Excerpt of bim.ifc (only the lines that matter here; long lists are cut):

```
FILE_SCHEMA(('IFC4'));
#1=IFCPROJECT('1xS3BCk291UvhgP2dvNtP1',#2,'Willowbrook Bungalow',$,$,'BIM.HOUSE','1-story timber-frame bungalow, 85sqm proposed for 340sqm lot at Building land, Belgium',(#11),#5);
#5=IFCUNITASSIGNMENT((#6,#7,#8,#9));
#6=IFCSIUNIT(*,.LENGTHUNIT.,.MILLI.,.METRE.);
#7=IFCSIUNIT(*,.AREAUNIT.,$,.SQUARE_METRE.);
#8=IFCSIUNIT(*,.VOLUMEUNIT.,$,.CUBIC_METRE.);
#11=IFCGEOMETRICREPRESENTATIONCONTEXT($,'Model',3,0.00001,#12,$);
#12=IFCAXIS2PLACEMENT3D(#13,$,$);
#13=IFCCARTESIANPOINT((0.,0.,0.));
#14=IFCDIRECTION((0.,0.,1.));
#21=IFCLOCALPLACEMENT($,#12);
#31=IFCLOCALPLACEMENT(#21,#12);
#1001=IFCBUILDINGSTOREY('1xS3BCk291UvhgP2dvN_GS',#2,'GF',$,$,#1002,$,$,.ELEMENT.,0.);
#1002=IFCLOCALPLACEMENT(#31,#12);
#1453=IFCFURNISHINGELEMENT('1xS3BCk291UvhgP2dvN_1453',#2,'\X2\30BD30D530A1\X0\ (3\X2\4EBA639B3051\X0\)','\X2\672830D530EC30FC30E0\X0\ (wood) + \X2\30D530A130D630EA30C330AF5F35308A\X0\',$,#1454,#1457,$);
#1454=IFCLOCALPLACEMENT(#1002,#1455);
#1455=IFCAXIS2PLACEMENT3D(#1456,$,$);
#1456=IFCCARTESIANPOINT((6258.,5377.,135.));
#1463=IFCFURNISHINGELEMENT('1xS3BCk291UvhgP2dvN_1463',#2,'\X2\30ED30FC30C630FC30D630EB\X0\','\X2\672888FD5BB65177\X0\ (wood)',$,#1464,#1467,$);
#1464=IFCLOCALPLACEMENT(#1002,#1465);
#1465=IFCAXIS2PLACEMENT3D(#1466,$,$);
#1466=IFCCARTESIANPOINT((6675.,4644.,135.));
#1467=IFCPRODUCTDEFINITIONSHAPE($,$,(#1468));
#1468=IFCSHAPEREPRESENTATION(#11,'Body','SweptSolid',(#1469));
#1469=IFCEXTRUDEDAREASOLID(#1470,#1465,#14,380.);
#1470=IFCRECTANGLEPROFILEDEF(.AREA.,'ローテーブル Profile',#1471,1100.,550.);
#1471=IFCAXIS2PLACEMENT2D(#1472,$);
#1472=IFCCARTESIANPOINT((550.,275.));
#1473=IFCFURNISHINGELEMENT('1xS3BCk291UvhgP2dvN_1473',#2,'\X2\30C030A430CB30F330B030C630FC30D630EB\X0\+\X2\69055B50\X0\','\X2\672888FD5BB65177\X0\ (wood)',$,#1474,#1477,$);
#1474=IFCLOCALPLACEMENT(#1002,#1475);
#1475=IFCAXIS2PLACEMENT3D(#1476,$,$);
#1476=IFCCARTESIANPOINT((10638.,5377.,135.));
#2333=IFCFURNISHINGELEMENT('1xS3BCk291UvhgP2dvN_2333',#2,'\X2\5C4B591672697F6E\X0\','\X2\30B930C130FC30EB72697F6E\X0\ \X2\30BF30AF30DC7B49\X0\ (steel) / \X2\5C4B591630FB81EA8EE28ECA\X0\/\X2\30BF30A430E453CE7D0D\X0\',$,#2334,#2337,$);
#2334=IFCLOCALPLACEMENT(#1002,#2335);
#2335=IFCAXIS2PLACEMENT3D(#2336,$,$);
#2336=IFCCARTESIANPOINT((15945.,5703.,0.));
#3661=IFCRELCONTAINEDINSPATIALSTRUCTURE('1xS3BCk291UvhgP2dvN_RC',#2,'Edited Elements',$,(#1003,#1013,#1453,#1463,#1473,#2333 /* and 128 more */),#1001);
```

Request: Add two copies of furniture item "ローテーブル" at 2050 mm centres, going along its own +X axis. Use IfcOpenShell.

```python
import ifcopenshell
import ifcopenshell.api.geometry
import ifcopenshell.api.root
import ifcopenshell.util.element
import ifcopenshell.util.placement
import ifcopenshell.util.unit

model = ifcopenshell.open("bim.ifc")
unit_scale = ifcopenshell.util.unit.calculate_unit_scale(model)


def reuse_history(source, copy):
    """copy_class also copies each property set's owner history, people and application; keep the originals."""
    for rel in copy.IsDefinedBy:
        if rel.is_a("IfcRelDefinesByProperties") and (history := rel.RelatingPropertyDefinition.OwnerHistory):
            rel.RelatingPropertyDefinition.OwnerHistory = source.OwnerHistory
            ifcopenshell.util.element.remove_deep2(model, history)


source = model.by_guid("1xS3BCk291UvhgP2dvN_1463")
base = ifcopenshell.util.placement.get_local_placement(source.ObjectPlacement)
step = base[:3, 0] * 2.05 / unit_scale

for i in range(1, 3):
    copy = ifcopenshell.api.root.copy_class(model, product=source)
    copy.Representation = ifcopenshell.util.element.copy_deep(
        model, source.Representation, exclude=["IfcGeometricRepresentationContext", "IfcRepresentationMap"]
    )
    reuse_history(source, copy)
    matrix = base.copy()
    matrix[:3, 3] += i * step
    print("added at", matrix[:3, 3].round(3) + 0.0)
    ifcopenshell.api.geometry.edit_object_placement(model, product=copy, matrix=matrix, is_si=False)

model.write("bim-out.ifc")
```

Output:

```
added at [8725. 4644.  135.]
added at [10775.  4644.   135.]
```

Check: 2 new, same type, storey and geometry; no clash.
